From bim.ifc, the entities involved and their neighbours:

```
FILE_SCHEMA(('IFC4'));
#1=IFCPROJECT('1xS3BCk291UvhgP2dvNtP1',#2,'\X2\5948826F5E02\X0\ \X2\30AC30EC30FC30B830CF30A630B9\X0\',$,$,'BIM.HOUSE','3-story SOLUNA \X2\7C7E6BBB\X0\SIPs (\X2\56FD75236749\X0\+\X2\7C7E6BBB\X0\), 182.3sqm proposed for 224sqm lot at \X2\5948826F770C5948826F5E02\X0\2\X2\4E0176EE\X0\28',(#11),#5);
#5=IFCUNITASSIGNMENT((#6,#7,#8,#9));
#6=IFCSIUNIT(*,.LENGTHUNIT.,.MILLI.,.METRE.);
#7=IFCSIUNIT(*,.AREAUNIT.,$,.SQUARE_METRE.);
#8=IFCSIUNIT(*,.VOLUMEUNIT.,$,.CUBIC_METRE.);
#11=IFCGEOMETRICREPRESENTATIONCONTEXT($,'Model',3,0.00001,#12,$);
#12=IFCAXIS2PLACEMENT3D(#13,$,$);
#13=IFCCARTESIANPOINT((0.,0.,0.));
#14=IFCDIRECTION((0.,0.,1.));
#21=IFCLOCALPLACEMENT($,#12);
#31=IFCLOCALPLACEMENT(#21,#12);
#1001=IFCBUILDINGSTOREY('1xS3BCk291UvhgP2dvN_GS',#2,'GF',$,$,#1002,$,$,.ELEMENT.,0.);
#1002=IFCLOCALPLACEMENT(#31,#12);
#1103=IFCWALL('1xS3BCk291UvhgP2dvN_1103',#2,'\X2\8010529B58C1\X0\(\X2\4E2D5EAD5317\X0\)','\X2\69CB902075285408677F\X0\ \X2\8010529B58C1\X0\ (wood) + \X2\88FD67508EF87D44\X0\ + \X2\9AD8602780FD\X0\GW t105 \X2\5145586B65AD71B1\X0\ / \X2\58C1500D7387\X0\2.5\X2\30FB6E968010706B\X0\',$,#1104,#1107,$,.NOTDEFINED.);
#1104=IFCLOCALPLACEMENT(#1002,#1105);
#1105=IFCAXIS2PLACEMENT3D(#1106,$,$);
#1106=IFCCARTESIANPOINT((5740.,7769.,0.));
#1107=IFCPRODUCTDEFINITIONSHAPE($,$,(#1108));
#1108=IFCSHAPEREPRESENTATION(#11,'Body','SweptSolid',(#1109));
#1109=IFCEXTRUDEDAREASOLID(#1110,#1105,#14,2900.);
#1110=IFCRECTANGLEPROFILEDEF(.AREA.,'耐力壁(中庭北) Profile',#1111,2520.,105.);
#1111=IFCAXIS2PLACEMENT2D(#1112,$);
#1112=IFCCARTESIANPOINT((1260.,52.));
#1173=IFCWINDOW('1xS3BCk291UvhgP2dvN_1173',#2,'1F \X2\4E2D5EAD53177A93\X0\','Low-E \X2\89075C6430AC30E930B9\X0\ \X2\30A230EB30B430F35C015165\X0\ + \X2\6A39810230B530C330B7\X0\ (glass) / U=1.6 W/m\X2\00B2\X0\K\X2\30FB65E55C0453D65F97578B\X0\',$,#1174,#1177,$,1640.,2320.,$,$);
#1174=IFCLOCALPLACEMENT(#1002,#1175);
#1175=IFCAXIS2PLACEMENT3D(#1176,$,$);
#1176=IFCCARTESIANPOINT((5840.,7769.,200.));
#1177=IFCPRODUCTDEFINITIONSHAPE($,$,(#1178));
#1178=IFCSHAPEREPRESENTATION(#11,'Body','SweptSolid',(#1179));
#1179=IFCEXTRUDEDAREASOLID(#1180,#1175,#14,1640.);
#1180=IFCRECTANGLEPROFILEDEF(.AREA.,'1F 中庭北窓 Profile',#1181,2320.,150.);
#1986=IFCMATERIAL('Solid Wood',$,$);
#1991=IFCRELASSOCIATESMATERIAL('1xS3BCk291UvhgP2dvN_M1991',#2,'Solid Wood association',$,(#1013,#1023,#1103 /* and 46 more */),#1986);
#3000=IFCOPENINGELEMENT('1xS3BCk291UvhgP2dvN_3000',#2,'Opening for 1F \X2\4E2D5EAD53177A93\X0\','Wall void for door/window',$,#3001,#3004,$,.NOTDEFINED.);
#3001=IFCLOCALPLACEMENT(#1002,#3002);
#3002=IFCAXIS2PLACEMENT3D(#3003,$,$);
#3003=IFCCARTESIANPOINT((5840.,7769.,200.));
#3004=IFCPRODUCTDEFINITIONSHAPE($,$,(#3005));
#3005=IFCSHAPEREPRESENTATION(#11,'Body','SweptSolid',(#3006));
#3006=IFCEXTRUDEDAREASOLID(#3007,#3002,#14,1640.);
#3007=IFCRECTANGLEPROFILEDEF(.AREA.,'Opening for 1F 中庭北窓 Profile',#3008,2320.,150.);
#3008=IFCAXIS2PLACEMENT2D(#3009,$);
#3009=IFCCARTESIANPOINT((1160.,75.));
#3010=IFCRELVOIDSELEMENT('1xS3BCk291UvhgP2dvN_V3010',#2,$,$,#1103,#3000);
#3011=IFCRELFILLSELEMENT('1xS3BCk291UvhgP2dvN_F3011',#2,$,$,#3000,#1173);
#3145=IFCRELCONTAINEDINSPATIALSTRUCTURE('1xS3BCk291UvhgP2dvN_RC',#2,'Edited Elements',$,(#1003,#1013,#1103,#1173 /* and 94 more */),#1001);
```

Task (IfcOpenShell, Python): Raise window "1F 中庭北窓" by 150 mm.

```python
import numpy as np
import ifcopenshell
import ifcopenshell.api.geometry
import ifcopenshell.util.placement
import ifcopenshell.util.unit

model = ifcopenshell.open("bim.ifc")
unit_scale = ifcopenshell.util.unit.calculate_unit_scale(model)

window = model.by_guid("1xS3BCk291UvhgP2dvN_1173")
opening = window.FillsVoids[0].RelatingOpeningElement
dz = 150.0

shift = np.array([0.0, 0.0, dz])
# The window is not placed relative to its opening, so move both.
for product in (opening, window):
    matrix = ifcopenshell.util.placement.get_local_placement(product.ObjectPlacement)
    matrix[:3, 3] += shift
    ifcopenshell.api.geometry.edit_object_placement(model, product=product, matrix=matrix, is_si=False)

print(f"moved by {dz * unit_scale:+.3f} m")

model.write("bim_v2.ifc")
```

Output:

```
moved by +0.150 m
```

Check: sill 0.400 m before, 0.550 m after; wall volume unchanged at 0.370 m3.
